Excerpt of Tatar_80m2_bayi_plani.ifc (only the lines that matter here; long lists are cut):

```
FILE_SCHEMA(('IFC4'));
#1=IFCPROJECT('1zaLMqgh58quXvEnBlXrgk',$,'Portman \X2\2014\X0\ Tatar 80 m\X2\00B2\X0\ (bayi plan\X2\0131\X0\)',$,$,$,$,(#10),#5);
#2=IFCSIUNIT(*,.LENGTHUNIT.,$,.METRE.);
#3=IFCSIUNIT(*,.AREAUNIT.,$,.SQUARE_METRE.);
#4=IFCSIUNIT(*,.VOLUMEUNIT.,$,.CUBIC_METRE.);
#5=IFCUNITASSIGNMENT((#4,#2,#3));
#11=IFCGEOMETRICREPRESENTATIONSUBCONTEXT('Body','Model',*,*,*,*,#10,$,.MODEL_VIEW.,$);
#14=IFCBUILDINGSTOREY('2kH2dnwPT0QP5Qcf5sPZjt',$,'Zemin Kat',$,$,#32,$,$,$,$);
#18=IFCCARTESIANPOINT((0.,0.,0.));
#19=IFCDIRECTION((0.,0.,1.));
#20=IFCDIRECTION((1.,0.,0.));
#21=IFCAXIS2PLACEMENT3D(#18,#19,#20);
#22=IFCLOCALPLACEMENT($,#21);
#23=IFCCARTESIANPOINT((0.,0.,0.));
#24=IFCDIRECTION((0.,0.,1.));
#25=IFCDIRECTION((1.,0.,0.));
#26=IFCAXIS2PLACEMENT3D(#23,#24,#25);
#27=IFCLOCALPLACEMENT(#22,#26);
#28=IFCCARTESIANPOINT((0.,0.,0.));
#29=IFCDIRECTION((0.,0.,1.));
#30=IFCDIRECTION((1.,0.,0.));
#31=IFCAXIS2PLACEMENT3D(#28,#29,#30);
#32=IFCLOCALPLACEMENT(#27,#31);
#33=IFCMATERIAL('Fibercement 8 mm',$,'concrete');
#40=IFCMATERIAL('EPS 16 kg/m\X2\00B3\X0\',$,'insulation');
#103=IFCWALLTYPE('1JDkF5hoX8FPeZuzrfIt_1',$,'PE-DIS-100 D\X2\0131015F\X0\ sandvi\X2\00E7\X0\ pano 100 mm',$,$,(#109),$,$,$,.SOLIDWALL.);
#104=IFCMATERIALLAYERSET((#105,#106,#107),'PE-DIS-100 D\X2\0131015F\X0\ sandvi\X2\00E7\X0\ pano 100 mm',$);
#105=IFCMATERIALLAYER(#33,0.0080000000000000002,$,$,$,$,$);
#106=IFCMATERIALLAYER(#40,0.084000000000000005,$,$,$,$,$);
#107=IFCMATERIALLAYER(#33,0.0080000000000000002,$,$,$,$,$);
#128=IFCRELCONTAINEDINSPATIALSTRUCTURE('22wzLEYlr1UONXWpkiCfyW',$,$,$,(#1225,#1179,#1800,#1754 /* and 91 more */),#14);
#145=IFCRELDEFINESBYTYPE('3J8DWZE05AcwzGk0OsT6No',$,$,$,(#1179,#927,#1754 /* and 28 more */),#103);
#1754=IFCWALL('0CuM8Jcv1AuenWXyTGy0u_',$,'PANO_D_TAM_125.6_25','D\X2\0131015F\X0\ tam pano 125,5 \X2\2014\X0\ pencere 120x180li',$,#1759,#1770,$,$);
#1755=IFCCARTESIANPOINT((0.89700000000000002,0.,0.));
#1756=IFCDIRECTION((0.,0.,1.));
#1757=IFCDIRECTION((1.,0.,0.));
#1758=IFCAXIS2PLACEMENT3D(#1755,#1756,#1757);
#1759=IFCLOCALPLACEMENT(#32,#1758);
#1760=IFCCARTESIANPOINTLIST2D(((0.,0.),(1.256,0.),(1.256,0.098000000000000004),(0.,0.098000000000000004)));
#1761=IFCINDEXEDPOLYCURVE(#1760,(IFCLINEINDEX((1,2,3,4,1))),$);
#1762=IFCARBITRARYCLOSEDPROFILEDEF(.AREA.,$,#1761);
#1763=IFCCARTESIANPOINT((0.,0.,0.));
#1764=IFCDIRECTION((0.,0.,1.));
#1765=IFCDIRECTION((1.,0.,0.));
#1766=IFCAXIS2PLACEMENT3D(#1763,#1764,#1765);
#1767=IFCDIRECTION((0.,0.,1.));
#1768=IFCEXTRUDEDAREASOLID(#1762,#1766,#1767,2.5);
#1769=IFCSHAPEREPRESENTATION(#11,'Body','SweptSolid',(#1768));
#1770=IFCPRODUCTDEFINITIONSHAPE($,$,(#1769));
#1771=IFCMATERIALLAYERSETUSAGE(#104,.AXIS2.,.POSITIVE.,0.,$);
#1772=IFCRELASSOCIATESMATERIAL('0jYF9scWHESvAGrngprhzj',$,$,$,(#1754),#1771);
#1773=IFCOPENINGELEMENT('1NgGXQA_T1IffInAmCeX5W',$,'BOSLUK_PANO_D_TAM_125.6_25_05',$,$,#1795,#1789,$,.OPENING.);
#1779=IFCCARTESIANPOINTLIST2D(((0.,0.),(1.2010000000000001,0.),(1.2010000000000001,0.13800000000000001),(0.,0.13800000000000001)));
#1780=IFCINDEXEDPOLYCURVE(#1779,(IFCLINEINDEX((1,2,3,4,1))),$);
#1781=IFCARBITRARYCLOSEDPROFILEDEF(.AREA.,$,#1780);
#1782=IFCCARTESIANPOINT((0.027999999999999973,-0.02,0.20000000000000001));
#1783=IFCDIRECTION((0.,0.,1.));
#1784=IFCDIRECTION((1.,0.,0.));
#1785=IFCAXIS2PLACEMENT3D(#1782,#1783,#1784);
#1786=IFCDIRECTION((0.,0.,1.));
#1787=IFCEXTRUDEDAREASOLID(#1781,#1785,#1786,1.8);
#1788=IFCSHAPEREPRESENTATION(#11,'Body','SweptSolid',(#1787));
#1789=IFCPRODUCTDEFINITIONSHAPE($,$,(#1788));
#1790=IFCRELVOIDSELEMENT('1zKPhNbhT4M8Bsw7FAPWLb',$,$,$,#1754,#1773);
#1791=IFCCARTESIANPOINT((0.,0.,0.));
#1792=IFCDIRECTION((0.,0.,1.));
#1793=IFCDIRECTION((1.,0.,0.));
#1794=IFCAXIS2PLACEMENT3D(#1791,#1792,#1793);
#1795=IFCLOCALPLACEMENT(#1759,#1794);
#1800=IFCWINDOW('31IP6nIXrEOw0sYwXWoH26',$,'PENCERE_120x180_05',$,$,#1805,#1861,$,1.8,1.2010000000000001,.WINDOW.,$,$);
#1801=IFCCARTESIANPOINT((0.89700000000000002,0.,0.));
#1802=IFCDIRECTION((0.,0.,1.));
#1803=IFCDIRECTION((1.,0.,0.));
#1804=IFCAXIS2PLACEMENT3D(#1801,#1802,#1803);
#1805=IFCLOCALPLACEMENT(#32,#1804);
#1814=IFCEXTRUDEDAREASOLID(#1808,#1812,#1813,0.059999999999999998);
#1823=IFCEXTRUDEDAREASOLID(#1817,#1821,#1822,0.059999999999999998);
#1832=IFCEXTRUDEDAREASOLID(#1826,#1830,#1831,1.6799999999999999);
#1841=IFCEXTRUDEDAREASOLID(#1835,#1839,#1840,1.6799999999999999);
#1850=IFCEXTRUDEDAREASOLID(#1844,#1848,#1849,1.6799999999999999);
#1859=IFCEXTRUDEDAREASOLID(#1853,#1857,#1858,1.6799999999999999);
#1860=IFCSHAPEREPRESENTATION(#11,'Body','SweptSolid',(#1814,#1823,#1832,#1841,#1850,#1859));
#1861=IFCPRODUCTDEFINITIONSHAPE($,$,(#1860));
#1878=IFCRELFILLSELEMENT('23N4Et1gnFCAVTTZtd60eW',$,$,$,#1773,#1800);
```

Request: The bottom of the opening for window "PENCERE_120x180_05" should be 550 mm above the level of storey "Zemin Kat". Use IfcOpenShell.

```python
import numpy as np
import ifcopenshell
import ifcopenshell.api.geometry
import ifcopenshell.geom
import ifcopenshell.util.element
import ifcopenshell.util.placement
import ifcopenshell.util.shape
import ifcopenshell.util.unit

model = ifcopenshell.open("Tatar_80m2_bayi_plani.ifc")
unit_scale = ifcopenshell.util.unit.calculate_unit_scale(model)

window = model.by_guid("31IP6nIXrEOw0sYwXWoH26")
opening = window.FillsVoids[0].RelatingOpeningElement
storey = ifcopenshell.util.element.get_container(window, ifc_class="IfcBuildingStorey")
level = ifcopenshell.util.placement.get_local_placement(storey.ObjectPlacement)[2, 3]

# The opening's origin need not be at the sill, so measure its lowest point.
shape = ifcopenshell.geom.create_shape(ifcopenshell.geom.settings(), opening)
bottom = ifcopenshell.util.shape.get_shape_bottom_elevation(shape, shape.geometry) / unit_scale
dz = level + 0.55 - bottom

shift = np.array([0.0, 0.0, dz])
# The window is not placed relative to its opening, so move both.
for product in (opening, window):
    matrix = ifcopenshell.util.placement.get_local_placement(product.ObjectPlacement)
    matrix[:3, 3] += shift
    ifcopenshell.api.geometry.edit_object_placement(model, product=product, matrix=matrix, is_si=False)

print(f"moved by {dz * unit_scale:+.3f} m")

model.write("Tatar_80m2_bayi_plani_edited.ifc")
```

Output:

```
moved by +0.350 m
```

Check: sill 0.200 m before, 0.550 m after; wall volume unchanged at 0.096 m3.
